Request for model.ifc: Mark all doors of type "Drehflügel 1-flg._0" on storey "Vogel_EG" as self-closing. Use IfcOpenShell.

First a look at what the model holds.

```python
import ifcopenshell
import ifcopenshell.util.element

model = ifcopenshell.open("model.ifc")
print(model.schema)
storey = next(s for s in model.by_type("IfcBuildingStorey") if s.Name == "Vogel_EG")
doors = [e for e in ifcopenshell.util.element.get_decomposition(storey) if e.is_a("IfcDoor")]
seen = {}
for e in doors:
    element_type = ifcopenshell.util.element.get_type(e)
    key = (element_type.Name if element_type != e and element_type else None, ifcopenshell.util.element.get_pset(e, "Pset_DoorCommon", "SelfClosing"))
    seen[key] = seen.get(key, 0) + 1
for (name, value), count in sorted(seen.items(), key=str):
    print(count, "x", name, "|", value)
```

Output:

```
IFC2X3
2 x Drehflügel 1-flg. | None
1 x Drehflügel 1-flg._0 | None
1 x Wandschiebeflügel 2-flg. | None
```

```python
import ifcopenshell
import ifcopenshell.api.pset
import ifcopenshell.util.element

model = ifcopenshell.open("model.ifc")

storey = next(s for s in model.by_type("IfcBuildingStorey") if s.Name == "Vogel_EG")
doors = [e for e in ifcopenshell.util.element.get_decomposition(storey) if e.is_a("IfcDoor")]

count = 0
for e in doors:
    element_type = ifcopenshell.util.element.get_type(e)
    if element_type in (None, e) or element_type.Name != "Drehflügel 1-flg._0":
        continue
    # add_pset returns the element's existing set when there is one.
    pset = ifcopenshell.api.pset.add_pset(model, product=e, name="Pset_DoorCommon")
    ifcopenshell.api.pset.edit_pset(model, pset=pset, properties={"SelfClosing": True})
    count += 1

print(count, "doors updated")

model.write("model_rev.ifc")
```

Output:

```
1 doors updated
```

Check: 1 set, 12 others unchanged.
